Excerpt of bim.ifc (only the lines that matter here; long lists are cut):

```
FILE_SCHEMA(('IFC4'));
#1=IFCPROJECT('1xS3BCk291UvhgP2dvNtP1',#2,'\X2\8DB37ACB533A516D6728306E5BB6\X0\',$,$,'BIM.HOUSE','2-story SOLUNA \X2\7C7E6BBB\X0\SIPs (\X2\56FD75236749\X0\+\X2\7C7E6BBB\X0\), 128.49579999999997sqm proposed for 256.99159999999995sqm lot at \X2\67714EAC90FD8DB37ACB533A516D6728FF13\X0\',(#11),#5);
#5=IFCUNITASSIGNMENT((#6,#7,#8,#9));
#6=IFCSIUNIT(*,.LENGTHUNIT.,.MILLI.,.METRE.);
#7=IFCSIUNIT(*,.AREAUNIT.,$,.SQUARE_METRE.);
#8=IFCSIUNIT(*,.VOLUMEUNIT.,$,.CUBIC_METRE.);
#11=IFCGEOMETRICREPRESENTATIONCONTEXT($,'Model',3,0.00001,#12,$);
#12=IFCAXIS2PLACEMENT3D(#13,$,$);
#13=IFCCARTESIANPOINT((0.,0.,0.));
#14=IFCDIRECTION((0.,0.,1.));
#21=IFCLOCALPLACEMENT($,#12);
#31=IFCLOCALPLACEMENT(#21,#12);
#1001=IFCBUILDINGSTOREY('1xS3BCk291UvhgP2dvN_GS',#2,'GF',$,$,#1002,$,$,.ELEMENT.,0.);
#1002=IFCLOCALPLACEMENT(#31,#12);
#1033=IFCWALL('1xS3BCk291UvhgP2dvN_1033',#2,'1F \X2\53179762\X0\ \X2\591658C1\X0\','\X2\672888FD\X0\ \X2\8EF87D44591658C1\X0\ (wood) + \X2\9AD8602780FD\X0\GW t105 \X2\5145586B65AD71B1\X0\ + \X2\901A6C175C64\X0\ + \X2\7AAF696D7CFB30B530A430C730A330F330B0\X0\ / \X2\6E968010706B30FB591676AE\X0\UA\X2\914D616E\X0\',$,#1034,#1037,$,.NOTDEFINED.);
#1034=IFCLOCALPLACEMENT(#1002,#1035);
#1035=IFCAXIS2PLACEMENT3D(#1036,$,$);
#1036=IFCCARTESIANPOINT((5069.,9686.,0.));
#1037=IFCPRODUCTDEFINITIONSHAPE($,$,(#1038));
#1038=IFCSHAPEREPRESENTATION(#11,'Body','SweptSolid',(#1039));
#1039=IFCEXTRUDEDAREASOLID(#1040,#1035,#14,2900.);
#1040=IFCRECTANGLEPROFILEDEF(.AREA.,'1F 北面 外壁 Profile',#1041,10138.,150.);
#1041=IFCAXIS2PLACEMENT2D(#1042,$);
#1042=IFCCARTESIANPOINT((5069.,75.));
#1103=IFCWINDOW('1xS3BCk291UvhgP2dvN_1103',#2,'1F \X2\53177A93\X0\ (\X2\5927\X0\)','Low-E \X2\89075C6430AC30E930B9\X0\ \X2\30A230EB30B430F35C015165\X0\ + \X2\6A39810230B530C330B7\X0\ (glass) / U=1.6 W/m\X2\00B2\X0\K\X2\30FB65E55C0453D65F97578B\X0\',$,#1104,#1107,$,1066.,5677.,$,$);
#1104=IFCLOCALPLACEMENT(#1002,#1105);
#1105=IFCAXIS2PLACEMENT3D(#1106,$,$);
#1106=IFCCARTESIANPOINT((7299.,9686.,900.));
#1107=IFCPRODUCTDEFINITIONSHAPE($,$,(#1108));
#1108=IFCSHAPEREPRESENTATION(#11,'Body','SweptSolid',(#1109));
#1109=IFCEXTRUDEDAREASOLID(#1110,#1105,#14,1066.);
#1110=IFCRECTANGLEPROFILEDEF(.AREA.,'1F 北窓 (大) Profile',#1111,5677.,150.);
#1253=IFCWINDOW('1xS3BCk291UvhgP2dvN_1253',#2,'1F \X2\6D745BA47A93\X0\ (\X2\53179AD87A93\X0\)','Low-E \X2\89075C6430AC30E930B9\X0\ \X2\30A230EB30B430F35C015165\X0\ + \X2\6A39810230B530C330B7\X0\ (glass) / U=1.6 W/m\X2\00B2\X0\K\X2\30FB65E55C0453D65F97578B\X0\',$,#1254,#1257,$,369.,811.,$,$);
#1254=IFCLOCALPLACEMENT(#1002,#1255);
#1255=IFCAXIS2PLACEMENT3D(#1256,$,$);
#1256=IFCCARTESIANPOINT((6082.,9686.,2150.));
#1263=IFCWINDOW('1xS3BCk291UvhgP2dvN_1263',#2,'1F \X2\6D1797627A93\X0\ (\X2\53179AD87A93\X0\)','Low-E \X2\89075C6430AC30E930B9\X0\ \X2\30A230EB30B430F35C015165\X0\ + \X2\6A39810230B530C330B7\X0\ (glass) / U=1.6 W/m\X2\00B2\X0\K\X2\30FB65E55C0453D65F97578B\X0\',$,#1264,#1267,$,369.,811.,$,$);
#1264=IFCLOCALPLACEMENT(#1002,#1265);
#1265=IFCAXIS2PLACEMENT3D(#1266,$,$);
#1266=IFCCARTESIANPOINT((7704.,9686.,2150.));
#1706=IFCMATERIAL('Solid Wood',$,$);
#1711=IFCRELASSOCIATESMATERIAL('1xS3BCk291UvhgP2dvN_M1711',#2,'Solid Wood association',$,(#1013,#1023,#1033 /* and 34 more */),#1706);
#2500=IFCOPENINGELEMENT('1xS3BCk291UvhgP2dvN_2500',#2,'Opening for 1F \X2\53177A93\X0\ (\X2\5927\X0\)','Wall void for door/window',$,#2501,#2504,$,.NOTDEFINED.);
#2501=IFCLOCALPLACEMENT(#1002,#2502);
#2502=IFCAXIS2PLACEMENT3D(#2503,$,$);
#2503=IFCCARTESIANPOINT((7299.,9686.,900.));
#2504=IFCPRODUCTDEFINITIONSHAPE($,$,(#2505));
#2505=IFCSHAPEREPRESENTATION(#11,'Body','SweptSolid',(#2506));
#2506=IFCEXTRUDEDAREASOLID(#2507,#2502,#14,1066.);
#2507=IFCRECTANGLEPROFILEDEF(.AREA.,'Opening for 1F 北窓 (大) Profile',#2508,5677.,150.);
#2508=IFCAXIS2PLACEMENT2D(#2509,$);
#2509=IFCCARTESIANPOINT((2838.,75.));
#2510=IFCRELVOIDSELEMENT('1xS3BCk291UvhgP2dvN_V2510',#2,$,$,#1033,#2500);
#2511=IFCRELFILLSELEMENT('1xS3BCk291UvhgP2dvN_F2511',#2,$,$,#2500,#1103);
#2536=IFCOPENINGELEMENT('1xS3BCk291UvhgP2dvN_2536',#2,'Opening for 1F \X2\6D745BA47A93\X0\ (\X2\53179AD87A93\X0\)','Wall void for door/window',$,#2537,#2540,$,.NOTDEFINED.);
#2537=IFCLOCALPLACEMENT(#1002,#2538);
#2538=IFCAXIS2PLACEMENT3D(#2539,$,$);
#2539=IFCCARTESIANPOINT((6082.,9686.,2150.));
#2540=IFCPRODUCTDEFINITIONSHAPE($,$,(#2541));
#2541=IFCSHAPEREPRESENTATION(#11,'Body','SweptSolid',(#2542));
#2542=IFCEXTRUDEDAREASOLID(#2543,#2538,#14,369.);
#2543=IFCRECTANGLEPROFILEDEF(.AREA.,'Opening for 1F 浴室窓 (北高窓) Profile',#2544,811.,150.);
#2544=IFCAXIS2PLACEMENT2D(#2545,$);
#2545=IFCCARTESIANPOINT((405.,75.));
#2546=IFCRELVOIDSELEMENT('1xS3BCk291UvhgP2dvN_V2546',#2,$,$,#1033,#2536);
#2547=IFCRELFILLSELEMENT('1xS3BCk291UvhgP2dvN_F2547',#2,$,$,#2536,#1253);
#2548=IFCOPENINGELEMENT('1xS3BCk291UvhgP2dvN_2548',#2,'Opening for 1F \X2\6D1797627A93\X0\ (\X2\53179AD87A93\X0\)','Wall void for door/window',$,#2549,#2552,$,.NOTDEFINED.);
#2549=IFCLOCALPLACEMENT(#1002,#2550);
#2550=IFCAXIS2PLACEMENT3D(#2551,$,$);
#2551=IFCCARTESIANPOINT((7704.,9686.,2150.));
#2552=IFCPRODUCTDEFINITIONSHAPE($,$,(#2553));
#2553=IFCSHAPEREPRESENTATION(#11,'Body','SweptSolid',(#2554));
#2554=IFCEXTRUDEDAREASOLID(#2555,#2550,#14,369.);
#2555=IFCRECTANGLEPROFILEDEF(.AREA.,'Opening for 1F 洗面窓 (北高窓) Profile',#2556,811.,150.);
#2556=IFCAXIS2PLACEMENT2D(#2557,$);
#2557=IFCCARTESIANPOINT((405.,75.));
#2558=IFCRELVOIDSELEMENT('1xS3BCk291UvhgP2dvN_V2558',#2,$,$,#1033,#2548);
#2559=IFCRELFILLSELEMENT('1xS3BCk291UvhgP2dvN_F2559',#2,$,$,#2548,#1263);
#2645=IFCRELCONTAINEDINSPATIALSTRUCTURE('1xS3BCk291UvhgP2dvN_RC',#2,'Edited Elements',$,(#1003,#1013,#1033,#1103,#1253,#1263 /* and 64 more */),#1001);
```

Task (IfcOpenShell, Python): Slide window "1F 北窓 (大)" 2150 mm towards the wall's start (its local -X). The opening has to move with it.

```python
import ifcopenshell
import ifcopenshell.api.geometry
import ifcopenshell.util.placement

model = ifcopenshell.open("bim.ifc")

window = model.by_guid("1xS3BCk291UvhgP2dvN_1103")
opening = window.FillsVoids[0].RelatingOpeningElement
wall = opening.VoidsElements[0].RelatingBuildingElement

wall_matrix = ifcopenshell.util.placement.get_local_placement(wall.ObjectPlacement)
shift = wall_matrix[:3, 0] * -2150.0
before = ifcopenshell.util.placement.get_local_placement(window.ObjectPlacement)[:3, 3].copy()

# The window is not placed relative to its opening, so move both.
for product in (opening, window):
    matrix = ifcopenshell.util.placement.get_local_placement(product.ObjectPlacement)
    matrix[:3, 3] += shift
    ifcopenshell.api.geometry.edit_object_placement(model, product=product, matrix=matrix, is_si=False)

after = ifcopenshell.util.placement.get_local_placement(window.ObjectPlacement)[:3, 3]
print("window moved by", (after - before).round(3) + 0.0)

model.write("bim_updated.ifc")
```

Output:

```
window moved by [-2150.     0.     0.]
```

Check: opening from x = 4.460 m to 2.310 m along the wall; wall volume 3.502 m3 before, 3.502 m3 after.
